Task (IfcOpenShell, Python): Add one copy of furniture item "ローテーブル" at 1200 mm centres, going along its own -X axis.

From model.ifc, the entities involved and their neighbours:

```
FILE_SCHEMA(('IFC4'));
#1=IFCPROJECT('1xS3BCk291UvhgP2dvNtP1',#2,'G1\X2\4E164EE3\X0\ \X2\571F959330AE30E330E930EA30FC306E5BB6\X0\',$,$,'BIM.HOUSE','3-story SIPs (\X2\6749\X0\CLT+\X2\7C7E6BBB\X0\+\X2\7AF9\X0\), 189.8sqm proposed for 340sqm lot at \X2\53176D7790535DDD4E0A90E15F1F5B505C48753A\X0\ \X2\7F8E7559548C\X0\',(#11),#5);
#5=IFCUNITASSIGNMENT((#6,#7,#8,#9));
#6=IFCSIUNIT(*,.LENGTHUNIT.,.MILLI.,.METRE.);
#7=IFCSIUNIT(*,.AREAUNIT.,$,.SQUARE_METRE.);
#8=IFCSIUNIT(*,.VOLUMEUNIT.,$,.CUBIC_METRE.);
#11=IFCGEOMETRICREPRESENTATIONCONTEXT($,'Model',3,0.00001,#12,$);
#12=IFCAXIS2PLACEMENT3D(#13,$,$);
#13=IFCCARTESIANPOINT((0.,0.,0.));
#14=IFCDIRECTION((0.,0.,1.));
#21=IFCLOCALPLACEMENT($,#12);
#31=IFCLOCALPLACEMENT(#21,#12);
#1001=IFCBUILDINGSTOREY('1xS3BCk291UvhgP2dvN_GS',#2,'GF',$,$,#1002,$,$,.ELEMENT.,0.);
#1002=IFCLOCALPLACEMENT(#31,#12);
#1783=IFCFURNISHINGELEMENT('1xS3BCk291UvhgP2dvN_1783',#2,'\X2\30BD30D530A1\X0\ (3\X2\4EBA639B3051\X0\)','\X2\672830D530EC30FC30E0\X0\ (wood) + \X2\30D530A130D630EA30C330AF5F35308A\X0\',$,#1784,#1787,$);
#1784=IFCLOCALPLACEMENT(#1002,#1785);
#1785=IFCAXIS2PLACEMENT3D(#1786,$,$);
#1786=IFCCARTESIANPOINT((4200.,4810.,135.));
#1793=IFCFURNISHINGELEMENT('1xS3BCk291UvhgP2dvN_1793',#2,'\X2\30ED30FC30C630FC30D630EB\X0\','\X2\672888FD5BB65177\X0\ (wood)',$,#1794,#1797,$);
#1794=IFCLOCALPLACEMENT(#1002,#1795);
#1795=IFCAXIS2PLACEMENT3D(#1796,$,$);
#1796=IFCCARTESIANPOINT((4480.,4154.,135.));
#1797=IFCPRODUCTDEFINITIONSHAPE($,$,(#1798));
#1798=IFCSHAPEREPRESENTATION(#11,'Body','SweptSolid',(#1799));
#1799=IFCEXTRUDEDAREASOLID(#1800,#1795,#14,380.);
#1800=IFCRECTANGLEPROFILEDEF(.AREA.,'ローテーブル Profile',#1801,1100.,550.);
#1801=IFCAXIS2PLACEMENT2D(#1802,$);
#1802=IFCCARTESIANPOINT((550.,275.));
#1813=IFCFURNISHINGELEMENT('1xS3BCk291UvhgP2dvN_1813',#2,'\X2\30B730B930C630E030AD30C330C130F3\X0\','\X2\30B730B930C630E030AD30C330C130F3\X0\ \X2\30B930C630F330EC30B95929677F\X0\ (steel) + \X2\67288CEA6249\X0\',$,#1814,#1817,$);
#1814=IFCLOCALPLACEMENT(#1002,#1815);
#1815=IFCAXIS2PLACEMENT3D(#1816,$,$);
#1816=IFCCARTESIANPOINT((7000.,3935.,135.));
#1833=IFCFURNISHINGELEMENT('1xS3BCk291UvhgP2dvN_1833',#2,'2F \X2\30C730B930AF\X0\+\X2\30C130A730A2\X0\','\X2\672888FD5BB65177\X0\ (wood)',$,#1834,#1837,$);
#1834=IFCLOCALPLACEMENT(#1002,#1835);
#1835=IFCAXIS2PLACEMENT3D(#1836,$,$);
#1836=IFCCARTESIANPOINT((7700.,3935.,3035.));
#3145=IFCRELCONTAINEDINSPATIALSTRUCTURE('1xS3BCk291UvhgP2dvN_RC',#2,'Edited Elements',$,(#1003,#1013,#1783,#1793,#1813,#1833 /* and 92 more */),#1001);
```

```python
import ifcopenshell
import ifcopenshell.api.geometry
import ifcopenshell.api.root
import ifcopenshell.util.element
import ifcopenshell.util.placement
import ifcopenshell.util.unit

model = ifcopenshell.open("model.ifc")
unit_scale = ifcopenshell.util.unit.calculate_unit_scale(model)


def reuse_history(source, copy):
    """copy_class also copies each property set's owner history, people and application; keep the originals."""
    for rel in copy.IsDefinedBy:
        if rel.is_a("IfcRelDefinesByProperties") and (history := rel.RelatingPropertyDefinition.OwnerHistory):
            rel.RelatingPropertyDefinition.OwnerHistory = source.OwnerHistory
            ifcopenshell.util.element.remove_deep2(model, history)


source = model.by_guid("1xS3BCk291UvhgP2dvN_1793")
base = ifcopenshell.util.placement.get_local_placement(source.ObjectPlacement)
step = -base[:3, 0] * 1.2 / unit_scale

for i in range(1, 2):
    copy = ifcopenshell.api.root.copy_class(model, product=source)
    copy.Representation = ifcopenshell.util.element.copy_deep(
        model, source.Representation, exclude=["IfcGeometricRepresentationContext", "IfcRepresentationMap"]
    )
    reuse_history(source, copy)
    matrix = base.copy()
    matrix[:3, 3] += i * step
    print("added at", matrix[:3, 3].round(3) + 0.0)
    ifcopenshell.api.geometry.edit_object_placement(model, product=copy, matrix=matrix, is_si=False)

model.write("model_edited.ifc")
```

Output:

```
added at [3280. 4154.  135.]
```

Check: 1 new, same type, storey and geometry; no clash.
